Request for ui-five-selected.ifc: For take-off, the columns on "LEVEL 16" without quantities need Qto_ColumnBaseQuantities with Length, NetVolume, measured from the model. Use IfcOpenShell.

First a look at what the model holds.

```python
import ifcopenshell
import ifcopenshell.util.element
import ifcopenshell.util.unit

model = ifcopenshell.open("ui-five-selected.ifc")
print(model.schema)
for unit_type in ("LENGTHUNIT", "AREAUNIT", "VOLUMEUNIT"):
    print(unit_type, ifcopenshell.util.unit.calculate_unit_scale(model, unit_type))
storey = next(s for s in model.by_type("IfcBuildingStorey") if s.Name == "LEVEL 16")
columns = [e for e in ifcopenshell.util.element.get_decomposition(storey) if e.is_a("IfcColumn")]
for e in sorted(columns, key=lambda e: e.id()):
    print(e.id(), e.is_a(), e.Name, list(ifcopenshell.util.element.get_psets(e, qtos_only=True)), sep=" | ")
```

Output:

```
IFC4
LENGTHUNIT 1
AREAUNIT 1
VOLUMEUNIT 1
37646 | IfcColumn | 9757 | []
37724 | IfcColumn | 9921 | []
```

```python
import ifcopenshell
import ifcopenshell.api.pset
import ifcopenshell.geom
import ifcopenshell.util.element
import ifcopenshell.util.shape
import ifcopenshell.util.unit

model = ifcopenshell.open("ui-five-selected.ifc")
unit_scale = ifcopenshell.util.unit.calculate_unit_scale(model)
volume_scale = ifcopenshell.util.unit.calculate_unit_scale(model, "VOLUMEUNIT")
settings = ifcopenshell.geom.settings()

storey = next(s for s in model.by_type("IfcBuildingStorey") if s.Name == "LEVEL 16")
columns = [e for e in ifcopenshell.util.element.get_decomposition(storey) if e.is_a("IfcColumn")]

for e in sorted(columns, key=lambda e: e.id()):
    if ifcopenshell.util.element.get_psets(e, qtos_only=True, should_inherit=False):
        continue
    # Geometry comes back in metres, in the element's own axes.
    shape = ifcopenshell.geom.create_shape(settings, e)
    values = {
        "Length": ifcopenshell.util.shape.get_z(shape.geometry) / unit_scale,
        "NetVolume": ifcopenshell.util.shape.get_volume(shape.geometry) / volume_scale,
    }
    qto = ifcopenshell.api.pset.add_qto(model, product=e, name="Qto_ColumnBaseQuantities")
    ifcopenshell.api.pset.edit_qto(model, qto=qto, properties=values)
    print(e.id(), {k: round(v, 3) for k, v in values.items()})

model.write("ui-five-selected_rev.ifc")
```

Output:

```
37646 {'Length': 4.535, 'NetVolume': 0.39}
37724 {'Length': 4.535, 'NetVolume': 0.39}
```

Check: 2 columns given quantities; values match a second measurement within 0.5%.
